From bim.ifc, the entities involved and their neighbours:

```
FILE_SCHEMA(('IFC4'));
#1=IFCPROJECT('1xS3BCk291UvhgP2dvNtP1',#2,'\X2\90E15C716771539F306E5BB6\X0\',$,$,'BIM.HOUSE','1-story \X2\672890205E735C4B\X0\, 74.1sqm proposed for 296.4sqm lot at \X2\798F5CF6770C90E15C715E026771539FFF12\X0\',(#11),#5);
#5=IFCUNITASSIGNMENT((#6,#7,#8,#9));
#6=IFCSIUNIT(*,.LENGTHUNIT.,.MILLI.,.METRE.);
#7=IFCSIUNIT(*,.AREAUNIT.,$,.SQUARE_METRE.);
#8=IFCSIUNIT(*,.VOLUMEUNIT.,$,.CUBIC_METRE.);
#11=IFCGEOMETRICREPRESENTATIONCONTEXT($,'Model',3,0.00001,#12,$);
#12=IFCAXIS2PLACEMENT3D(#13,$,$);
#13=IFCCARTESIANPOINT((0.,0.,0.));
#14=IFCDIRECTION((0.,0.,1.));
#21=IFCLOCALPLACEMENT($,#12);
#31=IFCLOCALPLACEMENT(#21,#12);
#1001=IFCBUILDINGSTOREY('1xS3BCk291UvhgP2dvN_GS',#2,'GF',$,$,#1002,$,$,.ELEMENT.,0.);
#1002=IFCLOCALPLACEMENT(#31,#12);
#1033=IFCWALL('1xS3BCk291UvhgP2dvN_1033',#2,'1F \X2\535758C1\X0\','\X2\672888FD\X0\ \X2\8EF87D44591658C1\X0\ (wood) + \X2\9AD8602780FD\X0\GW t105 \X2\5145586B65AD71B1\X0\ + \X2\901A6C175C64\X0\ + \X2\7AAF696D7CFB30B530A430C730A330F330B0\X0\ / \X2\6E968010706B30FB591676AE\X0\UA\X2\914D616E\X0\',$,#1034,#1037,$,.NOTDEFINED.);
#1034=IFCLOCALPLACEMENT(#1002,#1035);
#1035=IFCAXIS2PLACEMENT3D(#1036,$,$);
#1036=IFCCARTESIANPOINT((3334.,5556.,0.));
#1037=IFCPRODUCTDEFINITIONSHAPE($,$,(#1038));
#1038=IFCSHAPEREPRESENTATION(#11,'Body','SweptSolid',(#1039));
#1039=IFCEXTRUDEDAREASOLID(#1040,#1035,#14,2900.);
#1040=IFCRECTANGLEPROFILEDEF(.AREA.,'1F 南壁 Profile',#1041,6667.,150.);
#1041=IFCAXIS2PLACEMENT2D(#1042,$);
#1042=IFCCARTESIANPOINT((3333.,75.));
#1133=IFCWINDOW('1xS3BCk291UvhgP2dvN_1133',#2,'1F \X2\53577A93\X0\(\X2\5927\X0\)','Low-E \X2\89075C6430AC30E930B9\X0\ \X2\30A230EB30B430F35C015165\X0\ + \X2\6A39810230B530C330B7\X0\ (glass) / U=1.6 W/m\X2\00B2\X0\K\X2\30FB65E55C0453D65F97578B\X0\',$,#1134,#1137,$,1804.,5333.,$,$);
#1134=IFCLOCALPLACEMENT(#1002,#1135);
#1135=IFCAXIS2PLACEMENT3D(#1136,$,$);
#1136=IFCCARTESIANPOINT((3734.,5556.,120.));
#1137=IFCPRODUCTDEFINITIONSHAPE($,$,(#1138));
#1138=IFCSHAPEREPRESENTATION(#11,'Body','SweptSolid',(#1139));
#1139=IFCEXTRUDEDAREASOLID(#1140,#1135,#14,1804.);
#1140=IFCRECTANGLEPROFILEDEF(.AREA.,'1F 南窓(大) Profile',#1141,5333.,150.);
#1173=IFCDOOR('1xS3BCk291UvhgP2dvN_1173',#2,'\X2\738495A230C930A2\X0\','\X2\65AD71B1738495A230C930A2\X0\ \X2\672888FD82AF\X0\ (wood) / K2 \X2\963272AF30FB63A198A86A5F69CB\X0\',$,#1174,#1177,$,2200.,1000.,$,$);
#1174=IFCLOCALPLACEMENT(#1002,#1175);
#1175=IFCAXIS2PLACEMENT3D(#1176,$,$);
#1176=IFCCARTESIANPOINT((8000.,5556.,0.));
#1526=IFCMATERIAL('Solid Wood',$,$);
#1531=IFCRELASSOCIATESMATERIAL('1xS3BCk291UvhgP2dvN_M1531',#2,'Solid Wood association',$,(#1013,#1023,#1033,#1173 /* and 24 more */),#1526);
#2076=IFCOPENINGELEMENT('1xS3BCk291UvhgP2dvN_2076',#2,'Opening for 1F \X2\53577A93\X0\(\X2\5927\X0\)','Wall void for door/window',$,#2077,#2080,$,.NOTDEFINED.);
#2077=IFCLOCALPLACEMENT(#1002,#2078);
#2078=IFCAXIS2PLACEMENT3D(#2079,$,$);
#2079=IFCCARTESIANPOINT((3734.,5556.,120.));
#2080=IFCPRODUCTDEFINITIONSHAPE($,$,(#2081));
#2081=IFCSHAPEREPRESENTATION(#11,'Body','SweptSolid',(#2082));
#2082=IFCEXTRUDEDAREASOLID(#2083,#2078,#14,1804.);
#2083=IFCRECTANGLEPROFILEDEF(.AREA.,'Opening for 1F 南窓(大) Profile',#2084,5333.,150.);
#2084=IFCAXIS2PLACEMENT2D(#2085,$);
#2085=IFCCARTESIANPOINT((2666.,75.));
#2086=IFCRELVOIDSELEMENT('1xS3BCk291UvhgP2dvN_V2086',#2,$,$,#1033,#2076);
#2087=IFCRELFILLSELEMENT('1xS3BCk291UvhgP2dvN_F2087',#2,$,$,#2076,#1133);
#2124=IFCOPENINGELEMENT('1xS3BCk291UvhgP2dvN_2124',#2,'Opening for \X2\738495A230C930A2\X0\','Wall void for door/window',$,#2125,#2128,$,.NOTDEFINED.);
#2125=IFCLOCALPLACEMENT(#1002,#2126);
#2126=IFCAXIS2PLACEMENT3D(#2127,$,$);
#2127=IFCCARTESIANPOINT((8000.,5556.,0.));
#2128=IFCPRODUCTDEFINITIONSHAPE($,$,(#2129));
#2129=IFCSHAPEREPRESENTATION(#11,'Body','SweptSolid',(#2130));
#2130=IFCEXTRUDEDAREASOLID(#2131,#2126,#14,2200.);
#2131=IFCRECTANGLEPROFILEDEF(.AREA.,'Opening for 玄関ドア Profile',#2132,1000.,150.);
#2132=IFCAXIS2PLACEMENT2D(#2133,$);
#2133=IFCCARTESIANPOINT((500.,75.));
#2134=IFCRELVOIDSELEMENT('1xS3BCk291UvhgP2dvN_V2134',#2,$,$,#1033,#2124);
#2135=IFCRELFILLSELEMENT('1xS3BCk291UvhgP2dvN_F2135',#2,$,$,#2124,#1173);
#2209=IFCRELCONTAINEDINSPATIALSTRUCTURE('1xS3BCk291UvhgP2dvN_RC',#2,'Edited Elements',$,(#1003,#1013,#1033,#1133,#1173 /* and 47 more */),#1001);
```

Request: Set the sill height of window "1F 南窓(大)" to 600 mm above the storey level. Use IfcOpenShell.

```python
import numpy as np
import ifcopenshell
import ifcopenshell.api.geometry
import ifcopenshell.geom
import ifcopenshell.util.element
import ifcopenshell.util.placement
import ifcopenshell.util.shape
import ifcopenshell.util.unit

model = ifcopenshell.open("bim.ifc")
unit_scale = ifcopenshell.util.unit.calculate_unit_scale(model)

window = model.by_guid("1xS3BCk291UvhgP2dvN_1133")
opening = window.FillsVoids[0].RelatingOpeningElement
storey = ifcopenshell.util.element.get_container(window, ifc_class="IfcBuildingStorey")
level = ifcopenshell.util.placement.get_local_placement(storey.ObjectPlacement)[2, 3]

# The opening's origin need not be at the sill, so measure its lowest point.
shape = ifcopenshell.geom.create_shape(ifcopenshell.geom.settings(), opening)
bottom = ifcopenshell.util.shape.get_shape_bottom_elevation(shape, shape.geometry) / unit_scale
dz = level + 600.0 - bottom

shift = np.array([0.0, 0.0, dz])
# The window is not placed relative to its opening, so move both.
for product in (opening, window):
    matrix = ifcopenshell.util.placement.get_local_placement(product.ObjectPlacement)
    matrix[:3, 3] += shift
    ifcopenshell.api.geometry.edit_object_placement(model, product=product, matrix=matrix, is_si=False)

print(f"moved by {dz * unit_scale:+.3f} m")

model.write("bim_rev.ifc")
```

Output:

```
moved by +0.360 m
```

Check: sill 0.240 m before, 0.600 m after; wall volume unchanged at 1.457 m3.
